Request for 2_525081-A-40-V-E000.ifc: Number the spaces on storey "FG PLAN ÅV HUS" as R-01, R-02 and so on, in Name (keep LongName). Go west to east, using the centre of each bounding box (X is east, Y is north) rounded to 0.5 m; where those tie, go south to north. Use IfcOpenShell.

First a look at what the model holds.

```python
import ifcopenshell
import ifcopenshell.util.element
import ifcopenshell.util.placement

model = ifcopenshell.open("2_525081-A-40-V-E000.ifc")
print(model.schema)
storey = next(s for s in model.by_type("IfcBuildingStorey") if s.Name == "FG PLAN ÅV HUS")
spaces = [e for e in ifcopenshell.util.element.get_decomposition(storey) if e.is_a("IfcSpace")]
for e in sorted(spaces, key=lambda e: e.id()):
    origin = ifcopenshell.util.placement.get_local_placement(e.ObjectPlacement)[:3, 3]
    print(e.id(), e.Name, e.LongName, origin.round(2) + 0.0, sep=" | ")
```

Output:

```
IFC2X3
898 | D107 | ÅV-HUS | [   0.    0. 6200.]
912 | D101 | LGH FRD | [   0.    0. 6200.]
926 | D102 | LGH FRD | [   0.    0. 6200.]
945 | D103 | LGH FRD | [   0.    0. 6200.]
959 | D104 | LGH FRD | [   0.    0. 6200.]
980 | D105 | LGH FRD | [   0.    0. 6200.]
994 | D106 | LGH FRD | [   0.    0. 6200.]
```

```python
import ifcopenshell
import ifcopenshell.geom
import ifcopenshell.util.element
import ifcopenshell.util.shape

model = ifcopenshell.open("2_525081-A-40-V-E000.ifc")
settings = ifcopenshell.geom.settings()
settings.set("use-world-coords", True)


def centre(element):
    shape = ifcopenshell.geom.create_shape(settings, element)
    return ifcopenshell.util.shape.get_bbox_centroid(shape.geometry)


storey = next(s for s in model.by_type("IfcBuildingStorey") if s.Name == "FG PLAN ÅV HUS")
spaces = [e for e in ifcopenshell.util.element.get_decomposition(storey) if e.is_a("IfcSpace")]

# Insertion points can sit at a corner or the storey origin, so sort by the geometry (in metres).
centres = {e: centre(e) for e in spaces}
spaces.sort(key=lambda e: (round(centres[e][0] / 0.5), centres[e][1]))

for i, e in enumerate(spaces, start=1):
    number = f"R-{i:02d}"
    e.Name = number
    print(e.id(), number)

model.write("2_525081-A-40-V-E000_v2.ifc")
```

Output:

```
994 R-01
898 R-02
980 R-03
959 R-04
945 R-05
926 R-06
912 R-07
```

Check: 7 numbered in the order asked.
